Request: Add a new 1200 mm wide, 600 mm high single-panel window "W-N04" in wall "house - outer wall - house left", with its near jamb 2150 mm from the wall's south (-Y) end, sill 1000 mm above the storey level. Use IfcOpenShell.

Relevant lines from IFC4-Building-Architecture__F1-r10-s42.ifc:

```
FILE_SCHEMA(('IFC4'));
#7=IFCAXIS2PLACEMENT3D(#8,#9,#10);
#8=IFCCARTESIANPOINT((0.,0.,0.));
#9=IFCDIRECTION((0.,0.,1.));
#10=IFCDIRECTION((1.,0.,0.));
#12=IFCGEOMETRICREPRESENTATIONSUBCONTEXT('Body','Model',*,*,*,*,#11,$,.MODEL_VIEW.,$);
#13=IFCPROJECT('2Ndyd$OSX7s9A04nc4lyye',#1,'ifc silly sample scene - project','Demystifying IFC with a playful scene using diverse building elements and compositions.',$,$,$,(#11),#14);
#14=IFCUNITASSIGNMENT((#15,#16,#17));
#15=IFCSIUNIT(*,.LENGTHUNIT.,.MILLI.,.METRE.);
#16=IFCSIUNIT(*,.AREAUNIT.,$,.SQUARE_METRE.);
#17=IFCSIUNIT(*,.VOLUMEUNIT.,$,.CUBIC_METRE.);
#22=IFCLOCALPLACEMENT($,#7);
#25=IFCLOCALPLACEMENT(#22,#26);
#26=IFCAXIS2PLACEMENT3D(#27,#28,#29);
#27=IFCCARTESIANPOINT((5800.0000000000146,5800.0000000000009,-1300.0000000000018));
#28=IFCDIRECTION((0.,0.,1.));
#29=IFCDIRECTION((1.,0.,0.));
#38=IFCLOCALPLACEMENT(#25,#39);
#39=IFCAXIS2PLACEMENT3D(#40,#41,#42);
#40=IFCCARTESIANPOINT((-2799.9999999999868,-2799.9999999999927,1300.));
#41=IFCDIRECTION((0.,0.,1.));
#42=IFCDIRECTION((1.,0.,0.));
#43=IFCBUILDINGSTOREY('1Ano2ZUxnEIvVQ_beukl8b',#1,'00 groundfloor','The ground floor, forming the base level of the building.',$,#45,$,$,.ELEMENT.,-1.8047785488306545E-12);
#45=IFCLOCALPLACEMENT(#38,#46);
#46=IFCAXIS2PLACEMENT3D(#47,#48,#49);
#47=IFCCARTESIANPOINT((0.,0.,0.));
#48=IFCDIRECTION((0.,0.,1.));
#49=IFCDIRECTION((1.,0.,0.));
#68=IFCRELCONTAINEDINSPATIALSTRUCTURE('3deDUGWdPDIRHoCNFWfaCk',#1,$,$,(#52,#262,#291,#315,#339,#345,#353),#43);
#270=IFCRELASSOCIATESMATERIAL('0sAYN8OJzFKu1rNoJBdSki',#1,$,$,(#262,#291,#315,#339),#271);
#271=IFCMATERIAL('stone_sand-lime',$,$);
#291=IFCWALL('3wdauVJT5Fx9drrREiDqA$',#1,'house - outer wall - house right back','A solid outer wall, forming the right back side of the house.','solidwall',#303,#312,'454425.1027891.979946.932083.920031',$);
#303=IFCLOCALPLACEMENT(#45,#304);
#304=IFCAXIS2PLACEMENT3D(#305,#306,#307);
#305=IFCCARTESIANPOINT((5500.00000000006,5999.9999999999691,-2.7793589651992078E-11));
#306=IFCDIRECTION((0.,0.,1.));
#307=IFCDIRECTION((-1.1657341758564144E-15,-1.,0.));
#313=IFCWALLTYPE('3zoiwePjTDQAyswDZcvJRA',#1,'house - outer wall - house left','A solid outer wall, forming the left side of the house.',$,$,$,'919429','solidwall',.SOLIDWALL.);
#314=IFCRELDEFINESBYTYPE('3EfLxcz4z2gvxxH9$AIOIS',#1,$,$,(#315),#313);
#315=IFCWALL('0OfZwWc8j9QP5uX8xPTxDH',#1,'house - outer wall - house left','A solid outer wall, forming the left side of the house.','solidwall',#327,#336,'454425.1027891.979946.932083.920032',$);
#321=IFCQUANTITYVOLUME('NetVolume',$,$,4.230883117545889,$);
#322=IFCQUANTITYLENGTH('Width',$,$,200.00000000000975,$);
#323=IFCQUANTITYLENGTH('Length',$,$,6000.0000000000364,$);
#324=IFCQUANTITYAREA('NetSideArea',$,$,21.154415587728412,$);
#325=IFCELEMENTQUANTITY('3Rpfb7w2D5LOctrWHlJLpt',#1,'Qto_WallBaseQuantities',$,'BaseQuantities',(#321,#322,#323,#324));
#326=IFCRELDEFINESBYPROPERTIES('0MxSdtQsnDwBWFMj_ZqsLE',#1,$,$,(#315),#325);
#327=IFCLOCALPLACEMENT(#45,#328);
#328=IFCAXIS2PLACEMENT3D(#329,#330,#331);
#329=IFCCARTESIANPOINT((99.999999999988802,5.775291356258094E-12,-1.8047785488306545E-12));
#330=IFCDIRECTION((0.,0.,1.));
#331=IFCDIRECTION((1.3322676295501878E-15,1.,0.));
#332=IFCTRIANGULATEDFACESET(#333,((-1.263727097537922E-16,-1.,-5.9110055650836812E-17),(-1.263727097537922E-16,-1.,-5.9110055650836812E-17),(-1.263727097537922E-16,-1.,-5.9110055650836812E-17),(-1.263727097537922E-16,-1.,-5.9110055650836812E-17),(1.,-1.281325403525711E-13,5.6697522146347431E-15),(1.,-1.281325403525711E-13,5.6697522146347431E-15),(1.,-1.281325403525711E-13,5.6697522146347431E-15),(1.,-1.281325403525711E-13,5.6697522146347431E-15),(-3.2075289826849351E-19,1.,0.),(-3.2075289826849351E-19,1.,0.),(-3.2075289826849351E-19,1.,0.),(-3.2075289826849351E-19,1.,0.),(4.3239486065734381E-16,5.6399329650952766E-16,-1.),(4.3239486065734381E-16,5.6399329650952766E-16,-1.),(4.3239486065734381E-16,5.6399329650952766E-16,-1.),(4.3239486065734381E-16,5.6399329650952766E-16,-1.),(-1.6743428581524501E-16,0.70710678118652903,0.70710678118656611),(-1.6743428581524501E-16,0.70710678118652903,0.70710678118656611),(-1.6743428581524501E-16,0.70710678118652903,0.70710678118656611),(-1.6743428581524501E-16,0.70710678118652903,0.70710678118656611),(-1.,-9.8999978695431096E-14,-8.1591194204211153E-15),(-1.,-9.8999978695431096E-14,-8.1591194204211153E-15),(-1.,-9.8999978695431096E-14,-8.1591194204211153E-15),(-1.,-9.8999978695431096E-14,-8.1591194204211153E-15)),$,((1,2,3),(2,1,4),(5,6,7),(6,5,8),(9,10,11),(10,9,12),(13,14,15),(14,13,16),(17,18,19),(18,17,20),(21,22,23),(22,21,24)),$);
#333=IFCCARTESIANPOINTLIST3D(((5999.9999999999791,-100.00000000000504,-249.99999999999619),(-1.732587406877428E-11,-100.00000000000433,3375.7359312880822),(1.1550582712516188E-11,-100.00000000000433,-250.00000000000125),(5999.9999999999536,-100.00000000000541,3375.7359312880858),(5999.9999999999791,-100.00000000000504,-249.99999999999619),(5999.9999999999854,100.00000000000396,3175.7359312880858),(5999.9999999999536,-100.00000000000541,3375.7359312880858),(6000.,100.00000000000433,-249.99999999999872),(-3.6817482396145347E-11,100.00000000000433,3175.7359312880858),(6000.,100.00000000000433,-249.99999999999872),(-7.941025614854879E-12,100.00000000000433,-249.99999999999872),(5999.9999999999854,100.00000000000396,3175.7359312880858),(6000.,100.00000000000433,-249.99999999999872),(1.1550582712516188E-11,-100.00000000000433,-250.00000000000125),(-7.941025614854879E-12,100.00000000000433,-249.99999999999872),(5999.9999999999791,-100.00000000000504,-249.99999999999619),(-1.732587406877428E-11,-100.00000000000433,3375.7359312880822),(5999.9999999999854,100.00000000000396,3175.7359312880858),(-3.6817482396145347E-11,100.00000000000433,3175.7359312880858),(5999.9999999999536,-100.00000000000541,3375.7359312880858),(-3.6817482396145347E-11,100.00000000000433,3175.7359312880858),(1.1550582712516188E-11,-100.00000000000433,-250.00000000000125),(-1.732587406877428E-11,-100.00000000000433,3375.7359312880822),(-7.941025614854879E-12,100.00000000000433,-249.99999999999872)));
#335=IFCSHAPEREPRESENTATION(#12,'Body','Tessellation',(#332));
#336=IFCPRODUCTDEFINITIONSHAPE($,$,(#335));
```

```python
import numpy as np
import ifcopenshell
import ifcopenshell.api.feature
import ifcopenshell.api.geometry
import ifcopenshell.api.pset
import ifcopenshell.api.root
import ifcopenshell.api.spatial
import ifcopenshell.geom
import ifcopenshell.util.element
import ifcopenshell.util.placement
import ifcopenshell.util.representation
import ifcopenshell.util.shape
import ifcopenshell.util.unit

model = ifcopenshell.open("IFC4-Building-Architecture__F1-r10-s42.ifc")
unit_scale = ifcopenshell.util.unit.calculate_unit_scale(model)
area_scale = ifcopenshell.util.unit.calculate_unit_scale(model, "AREAUNIT")
volume_scale = ifcopenshell.util.unit.calculate_unit_scale(model, "VOLUMEUNIT")
settings = ifcopenshell.geom.settings()


def volume(element):
    """Net volume in cubic metres, openings subtracted."""
    shape = ifcopenshell.geom.create_shape(settings, element)
    return ifcopenshell.util.shape.get_volume(shape.geometry)


wall = model.by_id(315)
storey = ifcopenshell.util.element.get_container(wall, ifc_class="IfcBuildingStorey")
context = ifcopenshell.util.representation.get_context(model, "Model", "Body", "MODEL_VIEW")
before = volume(wall)

width, height, from_end, sill = 1.2, 0.6, 2.15, 1  # metres

# The wall runs along its own X axis, and the end named is its -X end.
wall_shape = ifcopenshell.geom.create_shape(settings, wall)
x, y, z = ifcopenshell.util.shape.get_vertices(wall_shape.geometry).T
start = x.min() + from_end
face, thickness = float(y.min()), float(y.max() - y.min())
wall_matrix = ifcopenshell.util.placement.get_local_placement(wall.ObjectPlacement)
level = ifcopenshell.util.placement.get_local_placement(storey.ObjectPlacement)[2, 3]


def in_wall(x, y):
    """Placement at x, y metres in the wall's axes, at sill height."""
    matrix = wall_matrix.copy()
    matrix[:, 3] = wall_matrix @ np.array([x / unit_scale, y / unit_scale, 0.0, 1.0])
    matrix[2, 3] = level + sill / unit_scale
    return matrix


# Opening: a box that overshoots both wall faces by 50 mm.
opening = ifcopenshell.api.root.create_entity(model, ifc_class="IfcOpeningElement", predefined_type="OPENING")
box = ifcopenshell.api.geometry.add_wall_representation(
    model, context=context, length=width, height=height, thickness=thickness + 0.1
)
ifcopenshell.api.geometry.assign_representation(model, product=opening, representation=box)
ifcopenshell.api.geometry.edit_object_placement(model, product=opening, matrix=in_wall(start, face - 0.05), is_si=False)
ifcopenshell.api.feature.add_feature(model, feature=opening, element=wall)

window = ifcopenshell.api.root.create_entity(model, ifc_class="IfcWindow", name="W-N04", predefined_type="WINDOW")
window.OverallWidth, window.OverallHeight = width / unit_scale, height / unit_scale
window.PartitioningType = "SINGLE_PANEL"
body = ifcopenshell.api.geometry.add_window_representation(
    model,
    context=context,
    overall_width=window.OverallWidth,
    overall_height=window.OverallHeight,
    partition_type="SINGLE_PANEL",
)
ifcopenshell.api.geometry.assign_representation(model, product=window, representation=body)
ifcopenshell.api.spatial.assign_container(model, products=[window], relating_structure=storey)
ifcopenshell.api.feature.add_filling(model, opening=opening, element=window)

# Centre the window in the wall's thickness.
ifcopenshell.api.geometry.edit_object_placement(model, product=window, matrix=in_wall(start, face), is_si=False)
window_shape = ifcopenshell.geom.create_shape(settings, window)
depth = ifcopenshell.util.shape.get_vertices(window_shape.geometry)[:, 1]
offset = face + thickness / 2 - (depth.min() + depth.max()) / 2
ifcopenshell.api.geometry.edit_object_placement(model, product=window, matrix=in_wall(start, offset), is_si=False)

after = volume(wall)

# Update the wall's stored quantities.
qto = model.by_id(ifcopenshell.util.element.get_pset(wall, "Qto_WallBaseQuantities", should_inherit=False)["id"])
ifcopenshell.api.pset.edit_qto(model, qto=qto, properties={
    "NetVolume": after / volume_scale,
    "NetSideArea": after / thickness / area_scale,
})

print(f"wall volume {before:.3f} -> {after:.3f} m3")

model.write("IFC4-Building-Architecture__F1-r10-s42_edited.ifc")
```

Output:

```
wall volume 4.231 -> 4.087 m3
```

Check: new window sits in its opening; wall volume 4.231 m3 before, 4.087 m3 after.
